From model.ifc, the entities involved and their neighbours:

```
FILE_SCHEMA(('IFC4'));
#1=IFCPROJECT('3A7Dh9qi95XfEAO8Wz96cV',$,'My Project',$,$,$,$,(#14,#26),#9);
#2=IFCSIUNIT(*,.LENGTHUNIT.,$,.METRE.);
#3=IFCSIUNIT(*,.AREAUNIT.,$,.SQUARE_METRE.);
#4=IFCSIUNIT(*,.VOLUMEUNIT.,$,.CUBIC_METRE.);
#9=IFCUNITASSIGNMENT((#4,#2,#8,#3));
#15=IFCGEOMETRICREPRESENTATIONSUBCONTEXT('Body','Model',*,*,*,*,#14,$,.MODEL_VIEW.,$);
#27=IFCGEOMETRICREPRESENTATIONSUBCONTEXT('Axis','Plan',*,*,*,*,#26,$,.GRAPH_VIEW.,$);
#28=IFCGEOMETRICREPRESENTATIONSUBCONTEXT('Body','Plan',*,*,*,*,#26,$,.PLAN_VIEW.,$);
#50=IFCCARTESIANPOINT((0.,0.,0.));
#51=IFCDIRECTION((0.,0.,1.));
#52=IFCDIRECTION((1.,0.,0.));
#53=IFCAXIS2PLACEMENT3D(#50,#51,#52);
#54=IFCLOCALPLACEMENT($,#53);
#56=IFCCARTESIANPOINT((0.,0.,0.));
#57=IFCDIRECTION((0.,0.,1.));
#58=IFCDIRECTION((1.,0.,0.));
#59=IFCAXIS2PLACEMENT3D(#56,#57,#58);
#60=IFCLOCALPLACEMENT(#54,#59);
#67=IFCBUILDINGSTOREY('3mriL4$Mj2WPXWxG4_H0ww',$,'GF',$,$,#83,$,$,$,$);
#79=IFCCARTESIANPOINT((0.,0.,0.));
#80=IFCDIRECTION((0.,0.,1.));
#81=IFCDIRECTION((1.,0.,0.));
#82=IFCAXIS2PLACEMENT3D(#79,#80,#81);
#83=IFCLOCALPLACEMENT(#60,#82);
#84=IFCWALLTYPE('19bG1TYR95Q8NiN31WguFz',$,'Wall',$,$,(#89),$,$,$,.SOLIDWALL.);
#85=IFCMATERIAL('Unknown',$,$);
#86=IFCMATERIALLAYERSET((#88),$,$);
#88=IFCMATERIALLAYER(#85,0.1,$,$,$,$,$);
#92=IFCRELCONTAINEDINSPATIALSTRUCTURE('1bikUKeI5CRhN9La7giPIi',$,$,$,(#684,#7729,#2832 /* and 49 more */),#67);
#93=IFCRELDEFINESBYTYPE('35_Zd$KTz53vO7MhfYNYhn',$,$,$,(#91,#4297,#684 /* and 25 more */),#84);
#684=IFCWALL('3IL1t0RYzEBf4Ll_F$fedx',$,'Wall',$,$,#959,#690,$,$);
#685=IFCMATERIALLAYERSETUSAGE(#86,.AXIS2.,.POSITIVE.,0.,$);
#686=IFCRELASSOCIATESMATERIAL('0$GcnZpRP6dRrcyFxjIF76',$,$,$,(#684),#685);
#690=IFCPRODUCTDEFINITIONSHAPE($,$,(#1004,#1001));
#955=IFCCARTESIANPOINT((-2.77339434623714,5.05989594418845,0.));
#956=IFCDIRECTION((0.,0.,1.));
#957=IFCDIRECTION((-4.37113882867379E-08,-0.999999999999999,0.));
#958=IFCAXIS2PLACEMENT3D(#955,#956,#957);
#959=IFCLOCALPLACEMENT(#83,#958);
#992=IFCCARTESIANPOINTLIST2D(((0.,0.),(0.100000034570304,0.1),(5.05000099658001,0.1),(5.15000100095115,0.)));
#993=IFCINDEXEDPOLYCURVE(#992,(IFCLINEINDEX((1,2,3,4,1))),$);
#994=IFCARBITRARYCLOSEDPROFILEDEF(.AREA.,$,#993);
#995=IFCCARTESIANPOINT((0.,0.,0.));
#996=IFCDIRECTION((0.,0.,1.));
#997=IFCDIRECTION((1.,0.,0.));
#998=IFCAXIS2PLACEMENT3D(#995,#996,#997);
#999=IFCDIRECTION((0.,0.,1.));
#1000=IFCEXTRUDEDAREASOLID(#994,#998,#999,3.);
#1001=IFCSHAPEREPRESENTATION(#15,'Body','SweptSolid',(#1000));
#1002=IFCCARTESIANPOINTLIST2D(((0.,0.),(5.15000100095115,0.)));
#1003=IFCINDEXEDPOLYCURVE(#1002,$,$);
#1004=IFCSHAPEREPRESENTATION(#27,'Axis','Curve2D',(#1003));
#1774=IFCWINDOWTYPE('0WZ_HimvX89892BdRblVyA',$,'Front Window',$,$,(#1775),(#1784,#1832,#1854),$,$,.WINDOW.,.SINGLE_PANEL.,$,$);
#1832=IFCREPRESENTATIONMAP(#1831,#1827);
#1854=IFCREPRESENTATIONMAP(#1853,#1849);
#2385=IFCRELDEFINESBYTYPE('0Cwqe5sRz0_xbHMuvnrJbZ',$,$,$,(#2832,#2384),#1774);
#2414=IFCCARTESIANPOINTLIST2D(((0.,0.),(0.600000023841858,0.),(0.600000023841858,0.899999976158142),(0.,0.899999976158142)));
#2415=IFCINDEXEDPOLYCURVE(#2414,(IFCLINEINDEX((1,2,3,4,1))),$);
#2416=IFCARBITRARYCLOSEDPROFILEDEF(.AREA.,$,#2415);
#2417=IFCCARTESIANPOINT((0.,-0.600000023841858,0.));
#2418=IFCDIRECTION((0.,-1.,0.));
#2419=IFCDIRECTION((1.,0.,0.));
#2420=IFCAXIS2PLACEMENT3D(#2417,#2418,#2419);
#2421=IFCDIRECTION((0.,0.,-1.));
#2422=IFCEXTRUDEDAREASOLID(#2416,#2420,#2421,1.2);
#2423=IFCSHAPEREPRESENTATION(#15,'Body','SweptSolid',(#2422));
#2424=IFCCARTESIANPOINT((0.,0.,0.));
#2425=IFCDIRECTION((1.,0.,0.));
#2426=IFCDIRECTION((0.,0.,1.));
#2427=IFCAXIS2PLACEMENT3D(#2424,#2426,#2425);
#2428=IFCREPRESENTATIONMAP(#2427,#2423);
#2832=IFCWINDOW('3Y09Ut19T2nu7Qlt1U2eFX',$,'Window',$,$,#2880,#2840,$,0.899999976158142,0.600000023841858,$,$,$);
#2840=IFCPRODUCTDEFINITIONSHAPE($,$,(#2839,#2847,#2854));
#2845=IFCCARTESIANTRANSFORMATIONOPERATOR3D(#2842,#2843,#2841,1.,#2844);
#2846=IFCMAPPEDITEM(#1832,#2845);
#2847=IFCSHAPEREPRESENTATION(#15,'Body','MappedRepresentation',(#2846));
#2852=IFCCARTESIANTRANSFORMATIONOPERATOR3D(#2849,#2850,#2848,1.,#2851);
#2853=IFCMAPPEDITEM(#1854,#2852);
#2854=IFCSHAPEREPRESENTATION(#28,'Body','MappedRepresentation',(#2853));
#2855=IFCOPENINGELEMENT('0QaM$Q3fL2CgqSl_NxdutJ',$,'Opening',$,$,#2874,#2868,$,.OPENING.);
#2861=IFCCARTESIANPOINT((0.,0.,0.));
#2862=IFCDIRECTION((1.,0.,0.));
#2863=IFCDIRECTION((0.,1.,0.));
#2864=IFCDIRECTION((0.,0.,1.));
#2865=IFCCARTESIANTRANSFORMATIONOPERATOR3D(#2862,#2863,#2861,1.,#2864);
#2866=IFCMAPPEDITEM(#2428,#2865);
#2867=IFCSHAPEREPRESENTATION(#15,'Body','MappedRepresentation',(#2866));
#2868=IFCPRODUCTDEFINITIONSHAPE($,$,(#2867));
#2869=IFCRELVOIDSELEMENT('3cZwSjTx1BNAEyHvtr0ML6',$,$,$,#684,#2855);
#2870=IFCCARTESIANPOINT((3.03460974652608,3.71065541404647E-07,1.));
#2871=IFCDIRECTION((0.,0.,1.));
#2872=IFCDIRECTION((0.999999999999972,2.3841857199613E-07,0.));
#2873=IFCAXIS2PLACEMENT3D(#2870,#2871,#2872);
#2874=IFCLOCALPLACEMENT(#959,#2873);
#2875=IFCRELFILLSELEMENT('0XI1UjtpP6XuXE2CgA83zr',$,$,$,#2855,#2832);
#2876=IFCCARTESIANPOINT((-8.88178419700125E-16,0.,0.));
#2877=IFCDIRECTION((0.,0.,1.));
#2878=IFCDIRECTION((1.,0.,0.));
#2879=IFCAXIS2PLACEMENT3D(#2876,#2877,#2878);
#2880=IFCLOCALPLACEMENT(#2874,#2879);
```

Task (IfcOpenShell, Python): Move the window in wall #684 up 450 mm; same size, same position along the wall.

```python
import numpy as np
import ifcopenshell
import ifcopenshell.api.geometry
import ifcopenshell.util.placement
import ifcopenshell.util.unit

model = ifcopenshell.open("model.ifc")
unit_scale = ifcopenshell.util.unit.calculate_unit_scale(model)

window = model.by_guid("3Y09Ut19T2nu7Qlt1U2eFX")
opening = window.FillsVoids[0].RelatingOpeningElement
dz = 0.45 / unit_scale

shift = np.array([0.0, 0.0, dz])
# The window is placed relative to its opening, so it follows when the opening moves.
matrix = ifcopenshell.util.placement.get_local_placement(opening.ObjectPlacement)
matrix[:3, 3] += shift
ifcopenshell.api.geometry.edit_object_placement(
    model, product=opening, matrix=matrix, is_si=False, should_transform_children=True
)

print(f"moved by {dz * unit_scale:+.3f} m")

model.write("model_rev.ifc")
```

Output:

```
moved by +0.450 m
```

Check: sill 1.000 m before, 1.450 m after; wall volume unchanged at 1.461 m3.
